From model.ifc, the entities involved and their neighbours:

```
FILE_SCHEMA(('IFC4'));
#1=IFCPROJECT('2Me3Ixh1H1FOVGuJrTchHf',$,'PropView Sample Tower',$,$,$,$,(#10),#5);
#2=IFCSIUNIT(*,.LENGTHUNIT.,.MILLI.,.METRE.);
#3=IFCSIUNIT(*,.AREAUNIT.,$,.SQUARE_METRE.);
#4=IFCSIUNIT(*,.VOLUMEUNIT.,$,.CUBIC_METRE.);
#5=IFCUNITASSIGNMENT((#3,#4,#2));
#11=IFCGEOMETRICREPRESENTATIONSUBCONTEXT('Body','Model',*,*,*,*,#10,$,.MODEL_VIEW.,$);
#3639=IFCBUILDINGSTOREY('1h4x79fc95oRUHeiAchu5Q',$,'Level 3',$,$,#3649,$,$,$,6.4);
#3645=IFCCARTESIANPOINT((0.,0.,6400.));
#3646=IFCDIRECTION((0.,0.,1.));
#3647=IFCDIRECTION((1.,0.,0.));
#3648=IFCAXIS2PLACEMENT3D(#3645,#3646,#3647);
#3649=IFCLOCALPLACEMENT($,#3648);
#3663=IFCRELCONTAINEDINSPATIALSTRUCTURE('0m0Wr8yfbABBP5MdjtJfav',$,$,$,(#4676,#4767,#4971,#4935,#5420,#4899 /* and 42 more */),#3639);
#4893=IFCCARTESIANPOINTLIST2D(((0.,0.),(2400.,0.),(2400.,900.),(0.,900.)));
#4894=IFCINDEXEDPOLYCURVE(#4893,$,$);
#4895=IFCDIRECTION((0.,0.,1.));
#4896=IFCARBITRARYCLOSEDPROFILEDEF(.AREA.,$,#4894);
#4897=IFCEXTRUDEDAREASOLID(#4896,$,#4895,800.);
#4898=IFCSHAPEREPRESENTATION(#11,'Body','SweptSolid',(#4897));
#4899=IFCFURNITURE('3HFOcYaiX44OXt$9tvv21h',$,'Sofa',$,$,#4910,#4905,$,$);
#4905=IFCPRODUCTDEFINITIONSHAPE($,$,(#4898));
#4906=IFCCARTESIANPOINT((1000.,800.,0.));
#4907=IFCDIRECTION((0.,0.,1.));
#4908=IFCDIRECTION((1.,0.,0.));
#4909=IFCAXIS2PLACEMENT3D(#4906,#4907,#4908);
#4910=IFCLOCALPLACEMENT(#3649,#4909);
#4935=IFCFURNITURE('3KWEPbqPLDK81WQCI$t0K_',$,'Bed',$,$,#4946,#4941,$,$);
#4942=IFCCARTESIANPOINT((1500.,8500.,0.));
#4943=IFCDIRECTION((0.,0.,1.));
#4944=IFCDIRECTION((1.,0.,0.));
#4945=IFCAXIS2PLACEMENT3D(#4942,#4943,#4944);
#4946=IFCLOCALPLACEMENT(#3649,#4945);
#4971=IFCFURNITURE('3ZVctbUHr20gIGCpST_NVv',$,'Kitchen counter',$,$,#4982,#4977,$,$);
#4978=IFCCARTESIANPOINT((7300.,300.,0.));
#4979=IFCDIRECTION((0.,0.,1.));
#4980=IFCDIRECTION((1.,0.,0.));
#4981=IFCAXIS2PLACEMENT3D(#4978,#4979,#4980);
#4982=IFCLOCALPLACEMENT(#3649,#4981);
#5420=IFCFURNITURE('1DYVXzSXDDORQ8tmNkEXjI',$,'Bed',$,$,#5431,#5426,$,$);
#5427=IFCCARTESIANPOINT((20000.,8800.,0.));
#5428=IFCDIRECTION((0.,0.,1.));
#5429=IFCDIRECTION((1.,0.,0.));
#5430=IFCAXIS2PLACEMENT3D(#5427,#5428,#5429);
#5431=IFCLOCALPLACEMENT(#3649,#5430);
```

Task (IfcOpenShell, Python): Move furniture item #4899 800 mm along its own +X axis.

```python
import ifcopenshell
import ifcopenshell.api.geometry
import ifcopenshell.util.placement
import ifcopenshell.util.unit

model = ifcopenshell.open("model.ifc")
unit_scale = ifcopenshell.util.unit.calculate_unit_scale(model)

item = model.by_id(4899)
matrix = ifcopenshell.util.placement.get_local_placement(item.ObjectPlacement)
matrix[:3, 3] += matrix[:3, 0] * 0.8 / unit_scale
ifcopenshell.api.geometry.edit_object_placement(model, product=item, matrix=matrix, is_si=False)

print(ifcopenshell.util.placement.get_local_placement(item.ObjectPlacement).round(3) + 0.0)

model.write("model_v2.ifc")
```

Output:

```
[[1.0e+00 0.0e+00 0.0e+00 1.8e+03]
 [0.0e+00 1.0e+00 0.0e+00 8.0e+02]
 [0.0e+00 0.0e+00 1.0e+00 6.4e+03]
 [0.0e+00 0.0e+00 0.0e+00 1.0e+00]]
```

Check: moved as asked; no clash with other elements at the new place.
